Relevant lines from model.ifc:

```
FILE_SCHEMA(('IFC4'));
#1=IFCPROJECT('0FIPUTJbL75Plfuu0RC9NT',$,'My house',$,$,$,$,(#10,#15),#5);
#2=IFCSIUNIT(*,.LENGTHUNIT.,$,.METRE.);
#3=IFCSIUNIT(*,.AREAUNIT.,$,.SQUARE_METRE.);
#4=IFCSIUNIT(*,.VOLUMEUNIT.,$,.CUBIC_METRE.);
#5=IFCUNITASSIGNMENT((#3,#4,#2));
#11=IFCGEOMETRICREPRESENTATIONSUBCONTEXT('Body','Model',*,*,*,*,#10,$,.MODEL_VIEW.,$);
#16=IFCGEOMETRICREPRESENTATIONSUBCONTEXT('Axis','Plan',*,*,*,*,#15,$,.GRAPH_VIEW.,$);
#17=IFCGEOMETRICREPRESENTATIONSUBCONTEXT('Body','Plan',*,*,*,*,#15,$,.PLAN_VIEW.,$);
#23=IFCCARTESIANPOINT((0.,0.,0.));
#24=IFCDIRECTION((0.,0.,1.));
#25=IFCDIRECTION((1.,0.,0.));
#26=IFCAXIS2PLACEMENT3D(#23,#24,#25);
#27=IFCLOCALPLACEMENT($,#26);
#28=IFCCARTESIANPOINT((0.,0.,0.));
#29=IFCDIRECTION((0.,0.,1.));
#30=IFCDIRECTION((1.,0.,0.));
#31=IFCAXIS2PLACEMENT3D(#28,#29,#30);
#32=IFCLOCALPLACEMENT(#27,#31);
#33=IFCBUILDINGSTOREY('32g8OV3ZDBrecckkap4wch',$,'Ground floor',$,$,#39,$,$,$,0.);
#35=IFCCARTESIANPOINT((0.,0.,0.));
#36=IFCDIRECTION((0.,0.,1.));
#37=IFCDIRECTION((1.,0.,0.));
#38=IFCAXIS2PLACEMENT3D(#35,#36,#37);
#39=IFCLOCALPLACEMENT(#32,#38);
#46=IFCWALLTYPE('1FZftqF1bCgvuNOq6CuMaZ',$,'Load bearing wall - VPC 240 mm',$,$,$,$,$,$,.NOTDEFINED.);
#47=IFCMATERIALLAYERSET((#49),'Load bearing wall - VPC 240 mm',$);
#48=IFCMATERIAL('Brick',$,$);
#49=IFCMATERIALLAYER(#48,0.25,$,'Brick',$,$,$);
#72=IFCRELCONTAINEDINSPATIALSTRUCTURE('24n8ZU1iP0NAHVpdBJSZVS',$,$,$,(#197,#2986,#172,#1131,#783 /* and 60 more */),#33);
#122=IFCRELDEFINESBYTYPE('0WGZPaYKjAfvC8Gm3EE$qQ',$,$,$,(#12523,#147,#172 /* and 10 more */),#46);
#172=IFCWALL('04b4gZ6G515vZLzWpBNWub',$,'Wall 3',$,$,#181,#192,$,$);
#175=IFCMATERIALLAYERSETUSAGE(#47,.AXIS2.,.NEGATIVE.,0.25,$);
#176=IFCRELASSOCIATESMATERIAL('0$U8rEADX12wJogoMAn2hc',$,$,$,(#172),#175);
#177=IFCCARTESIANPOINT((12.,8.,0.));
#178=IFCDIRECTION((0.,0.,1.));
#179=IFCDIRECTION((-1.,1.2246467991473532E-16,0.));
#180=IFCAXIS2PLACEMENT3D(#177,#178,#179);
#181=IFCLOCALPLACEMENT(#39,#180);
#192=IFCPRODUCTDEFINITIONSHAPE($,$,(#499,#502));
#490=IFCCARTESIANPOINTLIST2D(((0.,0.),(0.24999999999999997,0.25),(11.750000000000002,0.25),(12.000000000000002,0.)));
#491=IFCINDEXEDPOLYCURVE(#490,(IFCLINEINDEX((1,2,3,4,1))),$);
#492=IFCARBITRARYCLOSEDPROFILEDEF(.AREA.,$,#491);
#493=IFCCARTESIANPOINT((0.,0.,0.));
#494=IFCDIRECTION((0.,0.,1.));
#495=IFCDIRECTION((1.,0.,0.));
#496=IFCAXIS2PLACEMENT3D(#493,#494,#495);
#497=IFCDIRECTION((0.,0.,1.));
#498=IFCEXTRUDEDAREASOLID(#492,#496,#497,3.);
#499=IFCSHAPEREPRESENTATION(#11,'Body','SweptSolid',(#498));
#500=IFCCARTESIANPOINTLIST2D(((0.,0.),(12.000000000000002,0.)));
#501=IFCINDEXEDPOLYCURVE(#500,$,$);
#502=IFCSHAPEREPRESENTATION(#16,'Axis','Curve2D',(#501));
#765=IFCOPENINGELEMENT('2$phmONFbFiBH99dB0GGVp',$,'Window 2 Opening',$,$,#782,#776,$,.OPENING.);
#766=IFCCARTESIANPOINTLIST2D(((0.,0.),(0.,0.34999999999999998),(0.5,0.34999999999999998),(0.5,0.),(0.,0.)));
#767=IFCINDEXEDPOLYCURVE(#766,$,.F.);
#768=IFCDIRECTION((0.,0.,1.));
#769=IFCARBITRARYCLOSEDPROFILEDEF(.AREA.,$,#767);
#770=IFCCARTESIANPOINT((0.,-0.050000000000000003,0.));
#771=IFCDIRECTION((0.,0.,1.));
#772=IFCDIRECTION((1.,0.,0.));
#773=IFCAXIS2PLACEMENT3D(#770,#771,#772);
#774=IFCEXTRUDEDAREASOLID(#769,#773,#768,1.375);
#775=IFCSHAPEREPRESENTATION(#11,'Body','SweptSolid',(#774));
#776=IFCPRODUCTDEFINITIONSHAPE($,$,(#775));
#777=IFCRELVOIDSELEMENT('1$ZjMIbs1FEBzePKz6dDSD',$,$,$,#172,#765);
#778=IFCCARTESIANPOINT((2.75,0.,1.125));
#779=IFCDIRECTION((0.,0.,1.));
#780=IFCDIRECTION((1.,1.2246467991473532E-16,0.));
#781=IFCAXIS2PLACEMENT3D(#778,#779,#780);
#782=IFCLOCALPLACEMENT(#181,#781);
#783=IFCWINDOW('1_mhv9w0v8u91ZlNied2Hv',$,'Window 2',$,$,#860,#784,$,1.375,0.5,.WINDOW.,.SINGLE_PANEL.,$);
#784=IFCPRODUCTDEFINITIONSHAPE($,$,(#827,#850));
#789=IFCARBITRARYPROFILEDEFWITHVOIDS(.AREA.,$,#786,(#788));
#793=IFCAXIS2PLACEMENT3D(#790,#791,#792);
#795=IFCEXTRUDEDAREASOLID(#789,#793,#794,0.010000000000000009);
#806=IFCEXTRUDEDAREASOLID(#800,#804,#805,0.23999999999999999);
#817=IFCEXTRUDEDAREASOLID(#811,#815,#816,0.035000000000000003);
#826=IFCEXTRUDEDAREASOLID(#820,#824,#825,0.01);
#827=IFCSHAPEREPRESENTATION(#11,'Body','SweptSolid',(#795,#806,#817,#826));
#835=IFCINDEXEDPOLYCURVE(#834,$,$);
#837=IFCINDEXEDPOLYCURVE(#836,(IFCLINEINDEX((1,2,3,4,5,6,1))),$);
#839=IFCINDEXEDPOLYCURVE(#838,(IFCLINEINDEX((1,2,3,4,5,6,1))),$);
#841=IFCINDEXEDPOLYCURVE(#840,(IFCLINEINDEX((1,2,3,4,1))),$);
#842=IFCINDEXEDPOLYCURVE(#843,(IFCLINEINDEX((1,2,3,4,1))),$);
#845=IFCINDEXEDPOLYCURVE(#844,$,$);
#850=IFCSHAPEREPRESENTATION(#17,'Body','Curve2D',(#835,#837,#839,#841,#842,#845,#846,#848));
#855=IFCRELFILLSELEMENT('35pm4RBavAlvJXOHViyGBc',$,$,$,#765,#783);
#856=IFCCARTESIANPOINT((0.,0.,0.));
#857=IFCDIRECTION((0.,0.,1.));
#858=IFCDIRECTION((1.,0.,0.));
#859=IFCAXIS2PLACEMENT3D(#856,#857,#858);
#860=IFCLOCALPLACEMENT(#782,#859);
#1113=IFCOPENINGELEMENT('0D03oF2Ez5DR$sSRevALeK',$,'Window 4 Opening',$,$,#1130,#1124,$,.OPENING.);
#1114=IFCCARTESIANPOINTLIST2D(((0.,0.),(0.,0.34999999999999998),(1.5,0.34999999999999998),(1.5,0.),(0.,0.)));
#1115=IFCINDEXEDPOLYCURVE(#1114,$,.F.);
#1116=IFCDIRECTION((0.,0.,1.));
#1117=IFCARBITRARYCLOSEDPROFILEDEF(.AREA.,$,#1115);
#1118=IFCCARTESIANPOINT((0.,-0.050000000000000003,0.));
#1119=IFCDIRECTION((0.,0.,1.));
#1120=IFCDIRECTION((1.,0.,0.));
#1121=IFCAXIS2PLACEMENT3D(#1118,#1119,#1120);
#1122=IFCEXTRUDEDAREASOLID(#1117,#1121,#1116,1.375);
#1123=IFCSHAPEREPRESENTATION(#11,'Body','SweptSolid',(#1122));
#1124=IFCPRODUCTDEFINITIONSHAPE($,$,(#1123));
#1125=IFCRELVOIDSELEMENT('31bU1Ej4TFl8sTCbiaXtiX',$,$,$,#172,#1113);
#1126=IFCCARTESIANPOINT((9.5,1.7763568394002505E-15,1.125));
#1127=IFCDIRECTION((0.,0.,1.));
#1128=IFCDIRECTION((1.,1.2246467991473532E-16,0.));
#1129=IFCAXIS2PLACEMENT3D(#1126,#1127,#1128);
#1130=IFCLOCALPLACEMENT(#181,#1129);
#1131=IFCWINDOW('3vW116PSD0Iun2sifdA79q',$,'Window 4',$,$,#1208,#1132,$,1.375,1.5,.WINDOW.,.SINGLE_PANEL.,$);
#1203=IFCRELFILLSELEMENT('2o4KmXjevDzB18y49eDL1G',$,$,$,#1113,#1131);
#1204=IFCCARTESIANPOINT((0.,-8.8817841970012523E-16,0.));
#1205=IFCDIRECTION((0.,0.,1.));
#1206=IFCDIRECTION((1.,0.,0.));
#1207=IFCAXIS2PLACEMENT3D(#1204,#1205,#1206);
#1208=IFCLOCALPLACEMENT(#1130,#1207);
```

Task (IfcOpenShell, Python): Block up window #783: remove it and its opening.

```python
import ifcopenshell
import ifcopenshell.api.feature
import ifcopenshell.api.root
import ifcopenshell.geom
import ifcopenshell.util.shape

model = ifcopenshell.open("model.ifc")
settings = ifcopenshell.geom.settings()


def volume(element):
    """Net volume in cubic metres, openings subtracted."""
    shape = ifcopenshell.geom.create_shape(settings, element)
    return ifcopenshell.util.shape.get_volume(shape.geometry)


window = model.by_id(783)
opening = window.FillsVoids[0].RelatingOpeningElement
wall = opening.VoidsElements[0].RelatingBuildingElement
before = volume(wall)

ifcopenshell.api.root.remove_product(model, product=window)
ifcopenshell.api.feature.remove_feature(model, feature=opening)

after = volume(wall)

print(f"wall volume {before:.3f} -> {after:.3f} m3")

model.write("model_edited.ifc")
```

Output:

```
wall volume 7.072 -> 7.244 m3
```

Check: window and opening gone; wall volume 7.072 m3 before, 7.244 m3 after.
